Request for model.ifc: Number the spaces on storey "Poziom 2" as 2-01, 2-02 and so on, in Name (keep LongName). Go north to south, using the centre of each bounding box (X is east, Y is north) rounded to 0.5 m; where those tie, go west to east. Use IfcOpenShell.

First a look at what the model holds.

```python
import ifcopenshell
import ifcopenshell.util.element
import ifcopenshell.util.placement

model = ifcopenshell.open("model.ifc")
print(model.schema)
storey = next(s for s in model.by_type("IfcBuildingStorey") if s.Name == "Poziom 2")
spaces = [e for e in ifcopenshell.util.element.get_decomposition(storey) if e.is_a("IfcSpace")]
for e in sorted(spaces, key=lambda e: e.id()):
    origin = ifcopenshell.util.placement.get_local_placement(e.ObjectPlacement)[:3, 3]
    print(e.id(), e.Name, e.LongName, origin.round(2) + 0.0, sep=" | ")
```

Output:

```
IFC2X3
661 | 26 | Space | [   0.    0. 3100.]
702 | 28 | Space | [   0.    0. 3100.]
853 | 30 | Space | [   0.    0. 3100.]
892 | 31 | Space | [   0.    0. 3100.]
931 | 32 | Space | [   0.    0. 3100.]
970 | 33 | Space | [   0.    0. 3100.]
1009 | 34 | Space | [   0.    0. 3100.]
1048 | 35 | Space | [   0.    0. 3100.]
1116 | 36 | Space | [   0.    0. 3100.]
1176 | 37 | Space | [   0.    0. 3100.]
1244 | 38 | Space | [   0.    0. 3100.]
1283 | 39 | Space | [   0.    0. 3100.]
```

```python
import ifcopenshell
import ifcopenshell.geom
import ifcopenshell.util.element
import ifcopenshell.util.shape

model = ifcopenshell.open("model.ifc")
settings = ifcopenshell.geom.settings()
settings.set("use-world-coords", True)


def centre(element):
    shape = ifcopenshell.geom.create_shape(settings, element)
    return ifcopenshell.util.shape.get_bbox_centroid(shape.geometry)


storey = next(s for s in model.by_type("IfcBuildingStorey") if s.Name == "Poziom 2")
spaces = [e for e in ifcopenshell.util.element.get_decomposition(storey) if e.is_a("IfcSpace")]

# Insertion points can sit at a corner or the storey origin, so sort by the geometry (in metres).
centres = {e: centre(e) for e in spaces}
spaces.sort(key=lambda e: (-round(centres[e][1] / 0.5), centres[e][0]))

for i, e in enumerate(spaces, start=1):
    number = f"2-{i:02d}"
    e.Name = number
    print(e.id(), number)

model.write("model-out.ifc")
```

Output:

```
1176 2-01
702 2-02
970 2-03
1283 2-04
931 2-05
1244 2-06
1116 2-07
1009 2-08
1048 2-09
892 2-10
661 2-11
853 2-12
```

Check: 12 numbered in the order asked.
